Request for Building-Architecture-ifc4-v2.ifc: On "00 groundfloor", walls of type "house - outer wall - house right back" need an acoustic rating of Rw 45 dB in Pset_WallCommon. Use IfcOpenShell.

First a look at what the model holds.

```python
import ifcopenshell
import ifcopenshell.util.element

model = ifcopenshell.open("Building-Architecture-ifc4-v2.ifc")
print(model.schema)
storey = next(s for s in model.by_type("IfcBuildingStorey") if s.Name == "00 groundfloor")
walls = [e for e in ifcopenshell.util.element.get_decomposition(storey) if e.is_a("IfcWall")]
seen = {}
for e in walls:
    element_type = ifcopenshell.util.element.get_type(e)
    key = (element_type.Name if element_type != e and element_type else None, ifcopenshell.util.element.get_pset(e, "Pset_WallCommon", "AcousticRating"))
    seen[key] = seen.get(key, 0) + 1
for (name, value), count in sorted(seen.items(), key=str):
    print(count, "x", name, "|", value)
```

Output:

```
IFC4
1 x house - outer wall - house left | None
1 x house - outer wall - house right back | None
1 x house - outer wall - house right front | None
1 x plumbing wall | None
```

```python
import ifcopenshell
import ifcopenshell.api.pset
import ifcopenshell.util.element

model = ifcopenshell.open("Building-Architecture-ifc4-v2.ifc")

storey = next(s for s in model.by_type("IfcBuildingStorey") if s.Name == "00 groundfloor")
walls = [e for e in ifcopenshell.util.element.get_decomposition(storey) if e.is_a("IfcWall")]

count = 0
for e in walls:
    element_type = ifcopenshell.util.element.get_type(e)
    if element_type in (None, e) or element_type.Name != "house - outer wall - house right back":
        continue
    # add_pset returns the element's existing set when there is one.
    pset = ifcopenshell.api.pset.add_pset(model, product=e, name="Pset_WallCommon")
    ifcopenshell.api.pset.edit_pset(model, pset=pset, properties={"AcousticRating": "Rw 45 dB"})
    count += 1

print(count, "walls updated")

model.write("Building-Architecture-ifc4-v2_updated.ifc")
```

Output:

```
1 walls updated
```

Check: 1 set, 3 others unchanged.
